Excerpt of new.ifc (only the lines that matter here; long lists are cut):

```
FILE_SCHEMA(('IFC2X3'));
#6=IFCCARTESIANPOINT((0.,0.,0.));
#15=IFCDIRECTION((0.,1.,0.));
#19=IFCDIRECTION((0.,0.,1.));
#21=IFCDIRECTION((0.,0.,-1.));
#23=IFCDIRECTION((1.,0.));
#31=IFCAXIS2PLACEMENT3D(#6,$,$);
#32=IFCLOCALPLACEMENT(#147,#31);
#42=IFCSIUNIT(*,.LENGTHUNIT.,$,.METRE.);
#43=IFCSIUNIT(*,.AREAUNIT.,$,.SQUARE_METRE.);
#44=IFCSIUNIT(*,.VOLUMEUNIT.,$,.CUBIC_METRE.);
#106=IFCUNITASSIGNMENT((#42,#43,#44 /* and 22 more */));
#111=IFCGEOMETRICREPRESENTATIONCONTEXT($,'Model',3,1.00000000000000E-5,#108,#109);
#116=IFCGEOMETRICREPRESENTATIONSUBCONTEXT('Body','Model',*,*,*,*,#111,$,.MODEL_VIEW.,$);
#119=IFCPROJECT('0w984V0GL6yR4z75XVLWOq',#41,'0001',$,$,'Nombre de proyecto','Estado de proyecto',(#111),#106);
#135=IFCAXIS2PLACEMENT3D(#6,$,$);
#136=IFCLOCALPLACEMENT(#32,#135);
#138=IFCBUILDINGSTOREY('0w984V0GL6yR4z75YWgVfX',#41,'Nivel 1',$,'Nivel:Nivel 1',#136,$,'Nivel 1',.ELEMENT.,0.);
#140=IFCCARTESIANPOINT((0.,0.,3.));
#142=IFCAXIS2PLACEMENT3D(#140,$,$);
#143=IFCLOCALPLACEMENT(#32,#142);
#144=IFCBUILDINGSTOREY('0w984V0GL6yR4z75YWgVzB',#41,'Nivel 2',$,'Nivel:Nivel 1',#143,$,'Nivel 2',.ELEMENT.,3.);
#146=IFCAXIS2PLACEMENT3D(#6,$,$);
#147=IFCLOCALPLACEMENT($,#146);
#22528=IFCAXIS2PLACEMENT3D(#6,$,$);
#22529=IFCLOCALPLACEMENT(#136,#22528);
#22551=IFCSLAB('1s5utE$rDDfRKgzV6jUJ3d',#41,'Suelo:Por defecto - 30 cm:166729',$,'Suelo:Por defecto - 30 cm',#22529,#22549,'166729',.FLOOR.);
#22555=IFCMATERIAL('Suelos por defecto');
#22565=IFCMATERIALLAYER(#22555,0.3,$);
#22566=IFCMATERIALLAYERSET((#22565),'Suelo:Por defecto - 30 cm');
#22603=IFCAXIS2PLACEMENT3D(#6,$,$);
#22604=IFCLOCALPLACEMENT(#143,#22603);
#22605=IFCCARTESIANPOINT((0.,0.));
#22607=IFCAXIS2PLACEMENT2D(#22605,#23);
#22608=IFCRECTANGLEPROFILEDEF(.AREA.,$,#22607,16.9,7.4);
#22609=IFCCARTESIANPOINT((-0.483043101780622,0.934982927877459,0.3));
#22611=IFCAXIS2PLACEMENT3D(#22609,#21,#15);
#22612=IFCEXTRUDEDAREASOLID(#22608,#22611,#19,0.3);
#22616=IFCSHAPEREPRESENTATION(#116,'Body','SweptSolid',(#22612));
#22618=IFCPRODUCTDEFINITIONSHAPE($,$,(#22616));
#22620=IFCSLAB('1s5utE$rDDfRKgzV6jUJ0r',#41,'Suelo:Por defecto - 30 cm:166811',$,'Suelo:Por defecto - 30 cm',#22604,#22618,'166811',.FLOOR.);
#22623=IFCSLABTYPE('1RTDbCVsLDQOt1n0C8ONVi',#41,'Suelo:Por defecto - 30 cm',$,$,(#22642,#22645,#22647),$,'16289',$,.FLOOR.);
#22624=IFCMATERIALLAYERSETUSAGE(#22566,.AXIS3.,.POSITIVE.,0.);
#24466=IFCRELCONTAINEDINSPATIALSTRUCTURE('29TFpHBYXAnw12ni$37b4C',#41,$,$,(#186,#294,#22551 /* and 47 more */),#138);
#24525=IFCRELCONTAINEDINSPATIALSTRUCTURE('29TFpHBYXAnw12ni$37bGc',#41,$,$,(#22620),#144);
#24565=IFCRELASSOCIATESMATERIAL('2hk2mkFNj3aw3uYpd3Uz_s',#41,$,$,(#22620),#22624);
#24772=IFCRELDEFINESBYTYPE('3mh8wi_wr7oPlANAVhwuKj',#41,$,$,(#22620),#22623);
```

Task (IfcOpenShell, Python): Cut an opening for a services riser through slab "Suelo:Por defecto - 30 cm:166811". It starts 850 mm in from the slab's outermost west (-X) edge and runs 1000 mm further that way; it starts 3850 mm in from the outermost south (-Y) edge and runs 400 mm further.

```python
import numpy as np
import ifcopenshell
import ifcopenshell.api.feature
import ifcopenshell.api.geometry
import ifcopenshell.api.root
import ifcopenshell.geom
import ifcopenshell.util.placement
import ifcopenshell.util.representation
import ifcopenshell.util.shape
import ifcopenshell.util.unit

model = ifcopenshell.open("new.ifc")
unit_scale = ifcopenshell.util.unit.calculate_unit_scale(model)
settings = ifcopenshell.geom.settings()


def volume(element):
    """Net volume in cubic metres, openings subtracted."""
    shape = ifcopenshell.geom.create_shape(settings, element)
    return ifcopenshell.util.shape.get_volume(shape.geometry)


slab = model.by_guid("1s5utE$rDDfRKgzV6jUJ0r")
before = volume(slab)

# Extent in the slab's own axes, in metres. The edges named are its -X and -Y sides.
slab_shape = ifcopenshell.geom.create_shape(settings, slab)
vertices = ifcopenshell.util.shape.get_vertices(slab_shape.geometry)
x_min, y_min, bottom = vertices.min(axis=0)
top = vertices[:, 2].max()

opening = ifcopenshell.api.root.create_entity(model, ifc_class="IfcOpeningElement", name="Services riser opening")
context = ifcopenshell.util.representation.get_context(model, "Model", "Body", "MODEL_VIEW")
width, depth = 1, 0.4
outline = [(0.0, 0.0), (width, 0.0), (width, depth), (0.0, depth), (0.0, 0.0)]
# Overshoot both faces by 50 mm so the cut is clean.
shape = ifcopenshell.api.geometry.add_slab_representation(
    model, context=context, depth=top - bottom + 0.1, polyline=outline
)
ifcopenshell.api.geometry.assign_representation(model, product=opening, representation=shape)

matrix = ifcopenshell.util.placement.get_local_placement(slab.ObjectPlacement)
matrix[:, 3] = matrix @ np.append(np.array([x_min + 0.85, y_min + 3.85, bottom - 0.05]) / unit_scale, 1.0)
ifcopenshell.api.geometry.edit_object_placement(model, product=opening, matrix=matrix, is_si=False)
ifcopenshell.api.feature.add_feature(model, feature=opening, element=slab)

after = volume(slab)

print(f"slab volume {before:.3f} -> {after:.3f} m3")

model.write("new_rev.ifc")
```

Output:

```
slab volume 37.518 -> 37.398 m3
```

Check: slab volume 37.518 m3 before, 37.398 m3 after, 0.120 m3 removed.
